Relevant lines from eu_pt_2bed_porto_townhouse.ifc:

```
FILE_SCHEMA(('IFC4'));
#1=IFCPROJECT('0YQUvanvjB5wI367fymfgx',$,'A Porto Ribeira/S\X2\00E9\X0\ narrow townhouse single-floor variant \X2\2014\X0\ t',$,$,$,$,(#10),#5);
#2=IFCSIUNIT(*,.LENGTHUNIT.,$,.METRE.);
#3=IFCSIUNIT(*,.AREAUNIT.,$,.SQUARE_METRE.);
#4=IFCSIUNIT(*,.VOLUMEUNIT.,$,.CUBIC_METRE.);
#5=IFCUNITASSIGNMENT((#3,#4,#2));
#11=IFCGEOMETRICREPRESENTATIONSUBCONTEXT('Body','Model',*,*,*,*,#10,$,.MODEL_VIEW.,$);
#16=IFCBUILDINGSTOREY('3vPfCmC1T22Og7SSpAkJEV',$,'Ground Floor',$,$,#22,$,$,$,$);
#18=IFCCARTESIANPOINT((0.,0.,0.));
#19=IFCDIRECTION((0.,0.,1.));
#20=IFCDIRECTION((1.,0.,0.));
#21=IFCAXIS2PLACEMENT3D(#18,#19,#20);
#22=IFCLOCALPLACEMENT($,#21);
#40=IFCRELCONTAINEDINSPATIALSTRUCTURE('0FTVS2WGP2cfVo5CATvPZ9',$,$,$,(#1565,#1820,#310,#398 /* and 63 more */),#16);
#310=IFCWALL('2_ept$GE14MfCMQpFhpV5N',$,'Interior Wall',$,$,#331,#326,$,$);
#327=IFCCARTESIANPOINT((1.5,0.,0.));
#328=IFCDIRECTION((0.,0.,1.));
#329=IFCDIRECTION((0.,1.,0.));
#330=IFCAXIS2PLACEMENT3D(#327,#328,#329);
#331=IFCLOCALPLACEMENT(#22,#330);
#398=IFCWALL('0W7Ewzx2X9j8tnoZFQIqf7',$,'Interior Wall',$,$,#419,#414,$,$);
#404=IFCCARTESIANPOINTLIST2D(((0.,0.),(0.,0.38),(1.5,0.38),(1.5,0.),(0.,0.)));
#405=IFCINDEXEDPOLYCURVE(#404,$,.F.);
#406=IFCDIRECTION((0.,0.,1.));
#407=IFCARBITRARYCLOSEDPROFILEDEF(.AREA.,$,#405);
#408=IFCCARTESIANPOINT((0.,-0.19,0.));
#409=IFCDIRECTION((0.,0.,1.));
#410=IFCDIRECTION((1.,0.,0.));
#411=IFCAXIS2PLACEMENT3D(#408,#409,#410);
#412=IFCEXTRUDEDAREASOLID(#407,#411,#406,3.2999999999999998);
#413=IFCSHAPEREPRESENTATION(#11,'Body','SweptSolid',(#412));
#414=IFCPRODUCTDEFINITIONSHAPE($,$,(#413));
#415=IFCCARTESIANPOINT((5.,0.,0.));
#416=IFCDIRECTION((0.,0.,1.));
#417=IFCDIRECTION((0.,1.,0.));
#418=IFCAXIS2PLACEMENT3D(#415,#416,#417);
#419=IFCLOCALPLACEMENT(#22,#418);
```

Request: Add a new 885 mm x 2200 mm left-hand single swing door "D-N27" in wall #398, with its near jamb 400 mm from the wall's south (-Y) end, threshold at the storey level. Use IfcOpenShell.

```python
import numpy as np
import ifcopenshell
import ifcopenshell.api.feature
import ifcopenshell.api.geometry
import ifcopenshell.api.root
import ifcopenshell.api.spatial
import ifcopenshell.geom
import ifcopenshell.util.element
import ifcopenshell.util.placement
import ifcopenshell.util.representation
import ifcopenshell.util.shape
import ifcopenshell.util.unit

model = ifcopenshell.open("eu_pt_2bed_porto_townhouse.ifc")
unit_scale = ifcopenshell.util.unit.calculate_unit_scale(model)
settings = ifcopenshell.geom.settings()


def volume(element):
    """Net volume in cubic metres, openings subtracted."""
    shape = ifcopenshell.geom.create_shape(settings, element)
    return ifcopenshell.util.shape.get_volume(shape.geometry)


wall = model.by_guid("0W7Ewzx2X9j8tnoZFQIqf7")
storey = ifcopenshell.util.element.get_container(wall, ifc_class="IfcBuildingStorey")
context = ifcopenshell.util.representation.get_context(model, "Model", "Body", "MODEL_VIEW")
before = volume(wall)

width, height, from_end, sill = 0.885, 2.2, 0.4, 0.0  # metres

# The wall runs along its own X axis, and the end named is its -X end.
wall_shape = ifcopenshell.geom.create_shape(settings, wall)
x, y, z = ifcopenshell.util.shape.get_vertices(wall_shape.geometry).T
start = x.min() + from_end
face, thickness = float(y.min()), float(y.max() - y.min())
wall_matrix = ifcopenshell.util.placement.get_local_placement(wall.ObjectPlacement)
level = ifcopenshell.util.placement.get_local_placement(storey.ObjectPlacement)[2, 3]


def in_wall(x, y):
    """Placement at x, y metres in the wall's axes, at sill height."""
    matrix = wall_matrix.copy()
    matrix[:, 3] = wall_matrix @ np.array([x / unit_scale, y / unit_scale, 0.0, 1.0])
    matrix[2, 3] = level + sill / unit_scale
    return matrix


# Opening: a box that overshoots both wall faces by 50 mm.
opening = ifcopenshell.api.root.create_entity(model, ifc_class="IfcOpeningElement", predefined_type="OPENING")
box = ifcopenshell.api.geometry.add_wall_representation(
    model, context=context, length=width, height=height, thickness=thickness + 0.1
)
ifcopenshell.api.geometry.assign_representation(model, product=opening, representation=box)
ifcopenshell.api.geometry.edit_object_placement(model, product=opening, matrix=in_wall(start, face - 0.05), is_si=False)
ifcopenshell.api.feature.add_feature(model, feature=opening, element=wall)

door = ifcopenshell.api.root.create_entity(model, ifc_class="IfcDoor", name="D-N27", predefined_type="DOOR")
door.OverallWidth, door.OverallHeight = width / unit_scale, height / unit_scale
door.OperationType = "SINGLE_SWING_LEFT"
body = ifcopenshell.api.geometry.add_door_representation(
    model,
    context=context,
    overall_width=door.OverallWidth,
    overall_height=door.OverallHeight,
    operation_type="SINGLE_SWING_LEFT",
    lining_properties={"LiningDepth": thickness / unit_scale, "ThresholdDepth": thickness / unit_scale},
)
ifcopenshell.api.geometry.assign_representation(model, product=door, representation=body)
ifcopenshell.api.spatial.assign_container(model, products=[door], relating_structure=storey)
ifcopenshell.api.feature.add_filling(model, opening=opening, element=door)

# The lining spans the wall, so the door starts at the wall face.
ifcopenshell.api.geometry.edit_object_placement(model, product=door, matrix=in_wall(start, face), is_si=False)

after = volume(wall)

print(f"wall volume {before:.3f} -> {after:.3f} m3")

model.write("eu_pt_2bed_porto_townhouse_rev.ifc")
```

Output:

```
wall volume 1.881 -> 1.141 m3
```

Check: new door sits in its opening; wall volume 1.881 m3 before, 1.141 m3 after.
